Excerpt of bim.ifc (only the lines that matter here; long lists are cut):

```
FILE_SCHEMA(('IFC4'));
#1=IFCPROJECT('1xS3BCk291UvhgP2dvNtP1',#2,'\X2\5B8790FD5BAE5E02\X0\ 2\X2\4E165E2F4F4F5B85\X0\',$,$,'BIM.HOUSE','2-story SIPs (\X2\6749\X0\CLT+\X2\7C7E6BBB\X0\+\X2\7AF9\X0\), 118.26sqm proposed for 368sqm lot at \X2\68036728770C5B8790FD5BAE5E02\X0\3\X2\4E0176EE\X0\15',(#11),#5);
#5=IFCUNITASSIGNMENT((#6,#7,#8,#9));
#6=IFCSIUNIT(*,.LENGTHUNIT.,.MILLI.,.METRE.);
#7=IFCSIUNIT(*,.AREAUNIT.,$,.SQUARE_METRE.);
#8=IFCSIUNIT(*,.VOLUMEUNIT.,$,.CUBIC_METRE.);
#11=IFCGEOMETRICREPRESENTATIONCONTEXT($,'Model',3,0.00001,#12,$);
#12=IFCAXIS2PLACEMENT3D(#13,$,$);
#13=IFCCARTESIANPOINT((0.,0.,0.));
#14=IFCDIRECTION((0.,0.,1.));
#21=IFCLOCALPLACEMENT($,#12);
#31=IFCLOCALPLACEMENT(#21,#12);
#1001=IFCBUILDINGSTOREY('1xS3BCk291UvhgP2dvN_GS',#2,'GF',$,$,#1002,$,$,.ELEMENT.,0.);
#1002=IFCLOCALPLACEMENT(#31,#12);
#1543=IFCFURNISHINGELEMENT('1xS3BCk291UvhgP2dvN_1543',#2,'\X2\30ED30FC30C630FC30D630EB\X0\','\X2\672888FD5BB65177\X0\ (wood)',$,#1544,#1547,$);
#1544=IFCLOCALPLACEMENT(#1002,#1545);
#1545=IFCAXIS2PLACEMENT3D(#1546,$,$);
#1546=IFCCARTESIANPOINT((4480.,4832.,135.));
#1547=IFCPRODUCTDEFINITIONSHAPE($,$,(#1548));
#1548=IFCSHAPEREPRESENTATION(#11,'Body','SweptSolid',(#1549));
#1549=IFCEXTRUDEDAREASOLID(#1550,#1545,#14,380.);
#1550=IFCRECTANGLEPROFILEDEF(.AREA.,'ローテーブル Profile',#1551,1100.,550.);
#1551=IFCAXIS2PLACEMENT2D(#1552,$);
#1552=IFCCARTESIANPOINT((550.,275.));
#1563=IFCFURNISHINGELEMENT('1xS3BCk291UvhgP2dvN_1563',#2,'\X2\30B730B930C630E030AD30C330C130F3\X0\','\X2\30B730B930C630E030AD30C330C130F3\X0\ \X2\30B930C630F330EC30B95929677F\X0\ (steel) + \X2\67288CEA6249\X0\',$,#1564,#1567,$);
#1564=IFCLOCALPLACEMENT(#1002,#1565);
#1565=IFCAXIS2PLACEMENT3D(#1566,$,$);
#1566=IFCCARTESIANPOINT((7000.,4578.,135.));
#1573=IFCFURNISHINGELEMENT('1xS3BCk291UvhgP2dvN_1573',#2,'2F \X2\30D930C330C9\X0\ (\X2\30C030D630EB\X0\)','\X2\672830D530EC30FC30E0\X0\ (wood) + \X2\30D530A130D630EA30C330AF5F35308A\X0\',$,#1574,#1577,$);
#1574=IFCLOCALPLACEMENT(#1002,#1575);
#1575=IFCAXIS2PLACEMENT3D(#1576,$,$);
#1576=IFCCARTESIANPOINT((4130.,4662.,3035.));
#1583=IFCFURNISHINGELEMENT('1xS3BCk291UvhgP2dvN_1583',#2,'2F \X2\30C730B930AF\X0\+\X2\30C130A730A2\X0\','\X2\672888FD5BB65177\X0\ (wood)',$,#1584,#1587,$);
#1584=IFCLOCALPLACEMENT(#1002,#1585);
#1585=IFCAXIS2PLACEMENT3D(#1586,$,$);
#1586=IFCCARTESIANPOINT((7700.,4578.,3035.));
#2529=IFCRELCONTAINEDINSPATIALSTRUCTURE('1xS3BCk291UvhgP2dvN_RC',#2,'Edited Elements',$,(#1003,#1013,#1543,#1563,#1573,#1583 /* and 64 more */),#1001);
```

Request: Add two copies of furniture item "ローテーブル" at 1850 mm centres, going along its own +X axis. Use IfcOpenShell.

```python
import ifcopenshell
import ifcopenshell.api.geometry
import ifcopenshell.api.root
import ifcopenshell.util.element
import ifcopenshell.util.placement

model = ifcopenshell.open("bim.ifc")


def reuse_history(source, copy):
    """copy_class also copies each property set's owner history, people and application; keep the originals."""
    for rel in copy.IsDefinedBy:
        if rel.is_a("IfcRelDefinesByProperties") and (history := rel.RelatingPropertyDefinition.OwnerHistory):
            rel.RelatingPropertyDefinition.OwnerHistory = source.OwnerHistory
            ifcopenshell.util.element.remove_deep2(model, history)


source = model.by_guid("1xS3BCk291UvhgP2dvN_1543")
base = ifcopenshell.util.placement.get_local_placement(source.ObjectPlacement)
step = base[:3, 0] * 1850.0

for i in range(1, 3):
    copy = ifcopenshell.api.root.copy_class(model, product=source)
    copy.Representation = ifcopenshell.util.element.copy_deep(
        model, source.Representation, exclude=["IfcGeometricRepresentationContext", "IfcRepresentationMap"]
    )
    reuse_history(source, copy)
    matrix = base.copy()
    matrix[:3, 3] += i * step
    print("added at", matrix[:3, 3].round(3) + 0.0)
    ifcopenshell.api.geometry.edit_object_placement(model, product=copy, matrix=matrix, is_si=False)

model.write("bim_v2.ifc")
```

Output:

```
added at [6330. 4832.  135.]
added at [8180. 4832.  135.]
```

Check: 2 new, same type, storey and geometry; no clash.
